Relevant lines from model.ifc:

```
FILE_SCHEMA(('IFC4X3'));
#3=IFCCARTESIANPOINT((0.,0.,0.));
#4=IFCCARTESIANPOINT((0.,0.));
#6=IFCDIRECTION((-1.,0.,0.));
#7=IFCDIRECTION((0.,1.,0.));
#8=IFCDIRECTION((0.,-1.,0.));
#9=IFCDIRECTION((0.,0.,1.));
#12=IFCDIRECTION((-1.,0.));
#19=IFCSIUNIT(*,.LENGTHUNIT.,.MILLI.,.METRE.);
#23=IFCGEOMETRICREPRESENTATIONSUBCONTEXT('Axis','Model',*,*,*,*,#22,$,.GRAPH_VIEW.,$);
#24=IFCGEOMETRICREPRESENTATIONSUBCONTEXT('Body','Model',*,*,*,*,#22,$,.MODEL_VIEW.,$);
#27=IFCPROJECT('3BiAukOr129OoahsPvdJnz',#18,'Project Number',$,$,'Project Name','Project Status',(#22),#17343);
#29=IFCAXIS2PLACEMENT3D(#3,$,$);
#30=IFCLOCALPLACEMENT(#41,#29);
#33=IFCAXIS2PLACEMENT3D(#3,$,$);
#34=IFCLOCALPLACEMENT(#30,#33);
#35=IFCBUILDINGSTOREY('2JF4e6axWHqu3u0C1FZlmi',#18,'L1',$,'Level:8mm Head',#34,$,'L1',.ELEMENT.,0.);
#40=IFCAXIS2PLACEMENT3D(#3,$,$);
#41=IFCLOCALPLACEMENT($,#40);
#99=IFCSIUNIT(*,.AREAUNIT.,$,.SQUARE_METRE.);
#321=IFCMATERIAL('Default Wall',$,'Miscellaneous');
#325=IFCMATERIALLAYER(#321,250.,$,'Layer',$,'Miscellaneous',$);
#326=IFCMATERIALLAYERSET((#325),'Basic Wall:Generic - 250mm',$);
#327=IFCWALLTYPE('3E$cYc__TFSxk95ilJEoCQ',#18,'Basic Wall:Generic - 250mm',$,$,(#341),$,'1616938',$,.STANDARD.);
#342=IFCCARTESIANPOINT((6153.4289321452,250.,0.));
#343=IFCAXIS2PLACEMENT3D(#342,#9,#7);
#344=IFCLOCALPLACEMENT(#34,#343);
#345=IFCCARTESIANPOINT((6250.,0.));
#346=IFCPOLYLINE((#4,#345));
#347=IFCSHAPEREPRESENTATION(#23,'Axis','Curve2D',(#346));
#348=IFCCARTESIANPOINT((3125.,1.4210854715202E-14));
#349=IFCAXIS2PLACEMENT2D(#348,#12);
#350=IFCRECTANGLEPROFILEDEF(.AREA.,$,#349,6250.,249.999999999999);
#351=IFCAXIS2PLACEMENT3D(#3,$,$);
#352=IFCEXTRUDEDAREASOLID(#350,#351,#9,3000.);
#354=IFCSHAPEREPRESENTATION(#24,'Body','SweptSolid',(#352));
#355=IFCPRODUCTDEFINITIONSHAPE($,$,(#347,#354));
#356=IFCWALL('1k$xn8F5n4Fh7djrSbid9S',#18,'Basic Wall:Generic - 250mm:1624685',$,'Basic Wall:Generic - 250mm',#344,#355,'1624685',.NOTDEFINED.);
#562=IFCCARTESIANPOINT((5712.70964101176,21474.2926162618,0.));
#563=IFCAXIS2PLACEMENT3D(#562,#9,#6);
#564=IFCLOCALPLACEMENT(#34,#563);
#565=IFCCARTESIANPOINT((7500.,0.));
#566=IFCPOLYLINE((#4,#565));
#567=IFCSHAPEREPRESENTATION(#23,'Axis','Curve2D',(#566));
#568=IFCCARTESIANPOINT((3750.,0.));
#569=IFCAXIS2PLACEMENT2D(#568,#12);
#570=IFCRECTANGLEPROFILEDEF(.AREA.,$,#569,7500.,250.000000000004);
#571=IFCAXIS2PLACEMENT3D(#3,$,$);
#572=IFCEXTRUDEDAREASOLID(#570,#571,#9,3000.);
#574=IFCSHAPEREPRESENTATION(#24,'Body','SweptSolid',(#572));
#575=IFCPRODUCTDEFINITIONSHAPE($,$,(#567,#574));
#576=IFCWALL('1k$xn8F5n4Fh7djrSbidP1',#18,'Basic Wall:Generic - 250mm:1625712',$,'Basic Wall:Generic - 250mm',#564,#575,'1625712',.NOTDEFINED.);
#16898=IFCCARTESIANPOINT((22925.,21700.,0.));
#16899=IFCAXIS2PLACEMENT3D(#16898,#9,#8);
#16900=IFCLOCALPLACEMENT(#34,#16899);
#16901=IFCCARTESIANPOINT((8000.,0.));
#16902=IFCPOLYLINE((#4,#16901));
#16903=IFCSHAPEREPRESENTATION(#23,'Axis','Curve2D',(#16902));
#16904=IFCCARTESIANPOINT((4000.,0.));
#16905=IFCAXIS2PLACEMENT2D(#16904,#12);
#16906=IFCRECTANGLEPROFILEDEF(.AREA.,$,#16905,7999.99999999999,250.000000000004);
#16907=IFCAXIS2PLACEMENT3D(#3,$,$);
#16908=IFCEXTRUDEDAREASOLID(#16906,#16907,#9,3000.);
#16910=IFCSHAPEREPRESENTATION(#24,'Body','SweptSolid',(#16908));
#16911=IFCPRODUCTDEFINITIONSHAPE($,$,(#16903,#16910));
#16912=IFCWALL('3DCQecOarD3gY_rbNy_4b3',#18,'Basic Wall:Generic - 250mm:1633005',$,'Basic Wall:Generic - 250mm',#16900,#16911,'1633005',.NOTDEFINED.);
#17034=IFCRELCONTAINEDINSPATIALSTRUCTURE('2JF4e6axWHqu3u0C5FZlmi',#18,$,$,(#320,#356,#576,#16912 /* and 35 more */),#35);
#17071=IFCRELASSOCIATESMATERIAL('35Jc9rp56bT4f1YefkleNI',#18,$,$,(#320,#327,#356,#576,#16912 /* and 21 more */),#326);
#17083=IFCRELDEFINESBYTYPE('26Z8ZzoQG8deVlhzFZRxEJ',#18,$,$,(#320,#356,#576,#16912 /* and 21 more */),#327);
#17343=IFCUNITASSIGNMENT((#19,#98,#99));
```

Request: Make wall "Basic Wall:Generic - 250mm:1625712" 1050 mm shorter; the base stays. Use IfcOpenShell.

```python
import ifcopenshell
import ifcopenshell.geom
import ifcopenshell.util.representation
import ifcopenshell.util.shape
import ifcopenshell.util.unit

model = ifcopenshell.open("model.ifc")
unit_scale = ifcopenshell.util.unit.calculate_unit_scale(model)
settings = ifcopenshell.geom.settings()


def volume(element):
    """Net volume in cubic metres, openings subtracted."""
    shape = ifcopenshell.geom.create_shape(settings, element)
    return ifcopenshell.util.shape.get_volume(shape.geometry)


wall = model.by_guid("1k$xn8F5n4Fh7djrSbidP1")
before = volume(wall)

body = ifcopenshell.util.representation.get_representation(wall, "Model", "Body")
solid = body.Items[0]
old_height = solid.Depth
solid.Depth -= 1.05 / unit_scale
after = volume(wall)

print(f"height {old_height:g} -> {solid.Depth:g}, volume {before:.3f} -> {after:.3f} m3")

model.write("model_v2.ifc")
```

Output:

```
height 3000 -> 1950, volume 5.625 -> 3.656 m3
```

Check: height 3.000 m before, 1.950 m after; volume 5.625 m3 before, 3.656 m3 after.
